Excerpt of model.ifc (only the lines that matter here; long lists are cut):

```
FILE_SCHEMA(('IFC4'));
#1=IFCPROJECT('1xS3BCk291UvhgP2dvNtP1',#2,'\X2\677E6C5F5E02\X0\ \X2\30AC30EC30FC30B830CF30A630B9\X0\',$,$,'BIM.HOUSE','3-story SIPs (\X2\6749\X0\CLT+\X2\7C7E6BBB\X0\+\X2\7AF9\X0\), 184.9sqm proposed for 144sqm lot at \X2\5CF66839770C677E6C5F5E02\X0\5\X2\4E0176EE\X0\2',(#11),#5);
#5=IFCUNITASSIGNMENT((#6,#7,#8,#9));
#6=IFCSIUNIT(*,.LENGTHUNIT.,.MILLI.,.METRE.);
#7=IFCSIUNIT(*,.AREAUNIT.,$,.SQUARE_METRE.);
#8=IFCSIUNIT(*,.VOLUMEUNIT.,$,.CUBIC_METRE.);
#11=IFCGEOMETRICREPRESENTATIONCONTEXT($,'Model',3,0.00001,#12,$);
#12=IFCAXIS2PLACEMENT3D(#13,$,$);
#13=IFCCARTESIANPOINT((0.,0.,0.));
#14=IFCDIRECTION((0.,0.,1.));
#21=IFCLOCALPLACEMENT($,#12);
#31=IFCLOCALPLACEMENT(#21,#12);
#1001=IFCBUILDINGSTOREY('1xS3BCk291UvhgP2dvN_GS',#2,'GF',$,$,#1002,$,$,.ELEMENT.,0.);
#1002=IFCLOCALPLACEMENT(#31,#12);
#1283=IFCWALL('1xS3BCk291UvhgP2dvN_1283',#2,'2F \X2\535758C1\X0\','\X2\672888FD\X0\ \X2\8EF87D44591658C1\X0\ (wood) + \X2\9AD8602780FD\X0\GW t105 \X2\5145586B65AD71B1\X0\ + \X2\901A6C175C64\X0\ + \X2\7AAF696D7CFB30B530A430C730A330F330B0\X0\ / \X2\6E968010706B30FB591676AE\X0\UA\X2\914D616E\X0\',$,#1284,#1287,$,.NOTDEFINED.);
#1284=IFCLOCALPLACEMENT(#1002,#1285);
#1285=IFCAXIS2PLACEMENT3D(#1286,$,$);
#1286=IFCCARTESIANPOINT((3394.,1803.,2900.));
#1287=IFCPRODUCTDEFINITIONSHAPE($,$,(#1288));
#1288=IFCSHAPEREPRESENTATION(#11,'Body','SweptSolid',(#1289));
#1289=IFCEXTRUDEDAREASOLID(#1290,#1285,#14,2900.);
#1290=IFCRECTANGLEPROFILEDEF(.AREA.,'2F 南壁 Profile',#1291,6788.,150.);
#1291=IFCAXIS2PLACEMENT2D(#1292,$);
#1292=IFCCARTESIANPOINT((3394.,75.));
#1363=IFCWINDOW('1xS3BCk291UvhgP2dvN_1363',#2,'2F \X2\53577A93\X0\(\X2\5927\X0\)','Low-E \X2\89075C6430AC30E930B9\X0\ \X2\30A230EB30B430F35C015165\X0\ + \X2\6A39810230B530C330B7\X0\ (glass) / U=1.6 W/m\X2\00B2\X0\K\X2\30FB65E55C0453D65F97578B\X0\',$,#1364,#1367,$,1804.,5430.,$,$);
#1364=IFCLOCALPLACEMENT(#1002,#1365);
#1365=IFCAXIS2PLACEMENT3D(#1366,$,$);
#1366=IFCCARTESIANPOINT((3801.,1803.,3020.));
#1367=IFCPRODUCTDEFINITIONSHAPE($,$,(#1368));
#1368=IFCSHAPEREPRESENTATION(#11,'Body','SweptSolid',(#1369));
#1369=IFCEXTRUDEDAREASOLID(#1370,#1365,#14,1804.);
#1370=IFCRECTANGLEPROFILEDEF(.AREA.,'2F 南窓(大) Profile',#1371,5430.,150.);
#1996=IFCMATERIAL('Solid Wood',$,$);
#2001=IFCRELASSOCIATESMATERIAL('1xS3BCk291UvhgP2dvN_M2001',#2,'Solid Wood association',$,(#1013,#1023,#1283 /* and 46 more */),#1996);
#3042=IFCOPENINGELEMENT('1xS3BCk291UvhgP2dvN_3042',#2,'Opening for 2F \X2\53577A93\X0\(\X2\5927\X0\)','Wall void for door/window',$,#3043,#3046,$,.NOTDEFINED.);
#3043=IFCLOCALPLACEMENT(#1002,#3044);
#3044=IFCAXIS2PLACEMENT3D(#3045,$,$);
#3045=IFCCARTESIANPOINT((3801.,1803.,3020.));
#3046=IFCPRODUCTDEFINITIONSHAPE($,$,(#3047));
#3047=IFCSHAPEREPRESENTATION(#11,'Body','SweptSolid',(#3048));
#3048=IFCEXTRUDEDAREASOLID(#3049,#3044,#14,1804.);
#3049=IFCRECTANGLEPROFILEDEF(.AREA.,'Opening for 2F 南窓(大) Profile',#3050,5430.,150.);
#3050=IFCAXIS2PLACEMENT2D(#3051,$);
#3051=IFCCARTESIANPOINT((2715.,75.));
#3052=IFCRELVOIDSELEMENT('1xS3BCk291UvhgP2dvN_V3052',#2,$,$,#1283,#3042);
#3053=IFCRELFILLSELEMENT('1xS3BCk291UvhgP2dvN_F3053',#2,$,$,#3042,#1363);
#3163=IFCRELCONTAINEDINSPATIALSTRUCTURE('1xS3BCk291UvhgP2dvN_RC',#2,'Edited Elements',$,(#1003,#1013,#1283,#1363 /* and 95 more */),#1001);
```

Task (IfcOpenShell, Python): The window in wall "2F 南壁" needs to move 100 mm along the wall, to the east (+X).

```python
import ifcopenshell
import ifcopenshell.api.geometry
import ifcopenshell.util.placement

model = ifcopenshell.open("model.ifc")

window = model.by_id(1363)
opening = window.FillsVoids[0].RelatingOpeningElement
wall = opening.VoidsElements[0].RelatingBuildingElement

wall_matrix = ifcopenshell.util.placement.get_local_placement(wall.ObjectPlacement)
shift = wall_matrix[:3, 0] * 100.0
before = ifcopenshell.util.placement.get_local_placement(window.ObjectPlacement)[:3, 3].copy()

# The window is not placed relative to its opening, so move both.
for product in (opening, window):
    matrix = ifcopenshell.util.placement.get_local_placement(product.ObjectPlacement)
    matrix[:3, 3] += shift
    ifcopenshell.api.geometry.edit_object_placement(model, product=product, matrix=matrix, is_si=False)

after = ifcopenshell.util.placement.get_local_placement(window.ObjectPlacement)[:3, 3]
print("window moved by", (after - before).round(3) + 0.0)

model.write("model-out.ifc")
```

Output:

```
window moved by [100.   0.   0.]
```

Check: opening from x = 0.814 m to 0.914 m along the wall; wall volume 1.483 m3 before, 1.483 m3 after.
